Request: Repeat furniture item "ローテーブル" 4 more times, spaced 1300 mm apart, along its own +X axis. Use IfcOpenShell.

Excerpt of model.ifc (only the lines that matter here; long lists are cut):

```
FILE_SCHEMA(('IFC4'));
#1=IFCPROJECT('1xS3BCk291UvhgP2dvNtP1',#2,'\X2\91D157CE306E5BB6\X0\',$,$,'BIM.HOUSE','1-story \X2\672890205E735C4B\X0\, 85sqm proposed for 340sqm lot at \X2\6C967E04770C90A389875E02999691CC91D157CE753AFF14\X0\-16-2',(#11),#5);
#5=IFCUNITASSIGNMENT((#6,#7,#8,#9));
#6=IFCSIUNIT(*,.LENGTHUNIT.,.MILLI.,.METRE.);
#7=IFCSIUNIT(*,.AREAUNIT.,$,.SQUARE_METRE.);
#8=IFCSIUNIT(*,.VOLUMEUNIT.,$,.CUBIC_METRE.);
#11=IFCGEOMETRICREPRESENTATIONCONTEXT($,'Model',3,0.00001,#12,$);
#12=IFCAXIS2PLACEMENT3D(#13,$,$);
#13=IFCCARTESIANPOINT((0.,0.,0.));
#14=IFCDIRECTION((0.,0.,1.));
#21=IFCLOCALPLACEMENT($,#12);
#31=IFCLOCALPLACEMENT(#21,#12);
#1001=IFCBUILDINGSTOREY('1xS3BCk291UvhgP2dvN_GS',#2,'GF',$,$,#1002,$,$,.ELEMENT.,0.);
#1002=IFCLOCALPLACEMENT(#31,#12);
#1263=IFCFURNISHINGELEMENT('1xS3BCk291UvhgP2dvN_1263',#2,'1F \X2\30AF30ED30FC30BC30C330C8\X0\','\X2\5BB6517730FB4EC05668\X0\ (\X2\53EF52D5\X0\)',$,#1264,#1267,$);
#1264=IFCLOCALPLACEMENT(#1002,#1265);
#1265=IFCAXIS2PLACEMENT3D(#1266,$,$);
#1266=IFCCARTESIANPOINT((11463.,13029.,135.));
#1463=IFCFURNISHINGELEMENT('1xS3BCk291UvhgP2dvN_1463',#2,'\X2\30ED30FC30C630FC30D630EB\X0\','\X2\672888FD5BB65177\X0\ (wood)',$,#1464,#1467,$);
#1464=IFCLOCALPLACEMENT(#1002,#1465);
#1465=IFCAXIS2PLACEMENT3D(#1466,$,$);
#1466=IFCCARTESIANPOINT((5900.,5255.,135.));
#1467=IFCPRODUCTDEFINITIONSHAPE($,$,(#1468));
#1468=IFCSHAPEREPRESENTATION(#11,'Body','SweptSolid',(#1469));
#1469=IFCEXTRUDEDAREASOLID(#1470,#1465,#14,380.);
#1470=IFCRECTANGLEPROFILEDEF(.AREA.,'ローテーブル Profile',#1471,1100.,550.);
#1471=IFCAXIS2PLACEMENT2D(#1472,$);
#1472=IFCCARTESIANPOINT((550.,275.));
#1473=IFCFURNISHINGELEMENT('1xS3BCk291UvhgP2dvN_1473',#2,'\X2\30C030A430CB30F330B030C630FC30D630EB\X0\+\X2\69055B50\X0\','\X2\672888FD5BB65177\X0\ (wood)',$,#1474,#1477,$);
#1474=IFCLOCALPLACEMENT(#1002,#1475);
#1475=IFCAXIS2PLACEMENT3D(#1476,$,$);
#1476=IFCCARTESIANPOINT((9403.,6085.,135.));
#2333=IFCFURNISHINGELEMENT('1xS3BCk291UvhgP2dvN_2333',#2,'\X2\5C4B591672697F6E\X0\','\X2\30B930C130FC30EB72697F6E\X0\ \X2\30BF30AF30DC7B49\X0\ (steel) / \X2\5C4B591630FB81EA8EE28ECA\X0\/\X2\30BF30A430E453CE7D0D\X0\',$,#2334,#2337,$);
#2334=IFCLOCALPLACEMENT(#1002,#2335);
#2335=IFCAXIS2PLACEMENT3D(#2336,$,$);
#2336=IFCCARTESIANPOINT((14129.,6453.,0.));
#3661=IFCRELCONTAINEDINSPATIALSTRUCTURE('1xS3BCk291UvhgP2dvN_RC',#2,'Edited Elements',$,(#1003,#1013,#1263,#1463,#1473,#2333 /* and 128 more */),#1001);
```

```python
import ifcopenshell
import ifcopenshell.api.geometry
import ifcopenshell.api.root
import ifcopenshell.util.element
import ifcopenshell.util.placement

model = ifcopenshell.open("model.ifc")


def reuse_history(source, copy):
    """copy_class also copies each property set's owner history, people and application; keep the originals."""
    for rel in copy.IsDefinedBy:
        if rel.is_a("IfcRelDefinesByProperties") and (history := rel.RelatingPropertyDefinition.OwnerHistory):
            rel.RelatingPropertyDefinition.OwnerHistory = source.OwnerHistory
            ifcopenshell.util.element.remove_deep2(model, history)


source = model.by_guid("1xS3BCk291UvhgP2dvN_1463")
base = ifcopenshell.util.placement.get_local_placement(source.ObjectPlacement)
step = base[:3, 0] * 1300.0

for i in range(1, 5):
    copy = ifcopenshell.api.root.copy_class(model, product=source)
    copy.Representation = ifcopenshell.util.element.copy_deep(
        model, source.Representation, exclude=["IfcGeometricRepresentationContext", "IfcRepresentationMap"]
    )
    reuse_history(source, copy)
    matrix = base.copy()
    matrix[:3, 3] += i * step
    print("added at", matrix[:3, 3].round(3) + 0.0)
    ifcopenshell.api.geometry.edit_object_placement(model, product=copy, matrix=matrix, is_si=False)

model.write("model_edited.ifc")
```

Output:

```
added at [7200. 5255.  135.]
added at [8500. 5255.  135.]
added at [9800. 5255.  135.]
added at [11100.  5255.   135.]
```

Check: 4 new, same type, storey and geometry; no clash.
